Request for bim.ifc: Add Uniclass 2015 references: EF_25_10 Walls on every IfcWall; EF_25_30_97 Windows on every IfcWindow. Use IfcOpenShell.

First a look at what the model holds.

```python
import ifcopenshell

model = ifcopenshell.open("bim.ifc")
print(model.schema)
print("classifications:", [c.Name for c in model.by_type("IfcClassification")])
for ifc_class in ("IfcDoor", "IfcRoof", "IfcStair", "IfcWall", "IfcWindow"):
    print(ifc_class, len(model.by_type(ifc_class)))
```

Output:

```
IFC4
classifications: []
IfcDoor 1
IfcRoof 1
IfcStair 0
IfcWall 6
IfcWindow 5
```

```python
import ifcopenshell
import ifcopenshell.api.classification

model = ifcopenshell.open("bim.ifc")

system = ifcopenshell.api.classification.add_classification(model, classification="Uniclass 2015")

codes = {
    "IfcWall": ("EF_25_10", "Walls"),
    "IfcWindow": ("EF_25_30_97", "Windows"),
}
for ifc_class, (code, name) in codes.items():
    products = model.by_type(ifc_class)
    ifcopenshell.api.classification.add_reference(
        model, products=products, classification=system, identification=code, name=name
    )
    print(code, len(products))

model.write("bim_edited.ifc")
```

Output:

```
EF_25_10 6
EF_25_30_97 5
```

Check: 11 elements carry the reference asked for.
